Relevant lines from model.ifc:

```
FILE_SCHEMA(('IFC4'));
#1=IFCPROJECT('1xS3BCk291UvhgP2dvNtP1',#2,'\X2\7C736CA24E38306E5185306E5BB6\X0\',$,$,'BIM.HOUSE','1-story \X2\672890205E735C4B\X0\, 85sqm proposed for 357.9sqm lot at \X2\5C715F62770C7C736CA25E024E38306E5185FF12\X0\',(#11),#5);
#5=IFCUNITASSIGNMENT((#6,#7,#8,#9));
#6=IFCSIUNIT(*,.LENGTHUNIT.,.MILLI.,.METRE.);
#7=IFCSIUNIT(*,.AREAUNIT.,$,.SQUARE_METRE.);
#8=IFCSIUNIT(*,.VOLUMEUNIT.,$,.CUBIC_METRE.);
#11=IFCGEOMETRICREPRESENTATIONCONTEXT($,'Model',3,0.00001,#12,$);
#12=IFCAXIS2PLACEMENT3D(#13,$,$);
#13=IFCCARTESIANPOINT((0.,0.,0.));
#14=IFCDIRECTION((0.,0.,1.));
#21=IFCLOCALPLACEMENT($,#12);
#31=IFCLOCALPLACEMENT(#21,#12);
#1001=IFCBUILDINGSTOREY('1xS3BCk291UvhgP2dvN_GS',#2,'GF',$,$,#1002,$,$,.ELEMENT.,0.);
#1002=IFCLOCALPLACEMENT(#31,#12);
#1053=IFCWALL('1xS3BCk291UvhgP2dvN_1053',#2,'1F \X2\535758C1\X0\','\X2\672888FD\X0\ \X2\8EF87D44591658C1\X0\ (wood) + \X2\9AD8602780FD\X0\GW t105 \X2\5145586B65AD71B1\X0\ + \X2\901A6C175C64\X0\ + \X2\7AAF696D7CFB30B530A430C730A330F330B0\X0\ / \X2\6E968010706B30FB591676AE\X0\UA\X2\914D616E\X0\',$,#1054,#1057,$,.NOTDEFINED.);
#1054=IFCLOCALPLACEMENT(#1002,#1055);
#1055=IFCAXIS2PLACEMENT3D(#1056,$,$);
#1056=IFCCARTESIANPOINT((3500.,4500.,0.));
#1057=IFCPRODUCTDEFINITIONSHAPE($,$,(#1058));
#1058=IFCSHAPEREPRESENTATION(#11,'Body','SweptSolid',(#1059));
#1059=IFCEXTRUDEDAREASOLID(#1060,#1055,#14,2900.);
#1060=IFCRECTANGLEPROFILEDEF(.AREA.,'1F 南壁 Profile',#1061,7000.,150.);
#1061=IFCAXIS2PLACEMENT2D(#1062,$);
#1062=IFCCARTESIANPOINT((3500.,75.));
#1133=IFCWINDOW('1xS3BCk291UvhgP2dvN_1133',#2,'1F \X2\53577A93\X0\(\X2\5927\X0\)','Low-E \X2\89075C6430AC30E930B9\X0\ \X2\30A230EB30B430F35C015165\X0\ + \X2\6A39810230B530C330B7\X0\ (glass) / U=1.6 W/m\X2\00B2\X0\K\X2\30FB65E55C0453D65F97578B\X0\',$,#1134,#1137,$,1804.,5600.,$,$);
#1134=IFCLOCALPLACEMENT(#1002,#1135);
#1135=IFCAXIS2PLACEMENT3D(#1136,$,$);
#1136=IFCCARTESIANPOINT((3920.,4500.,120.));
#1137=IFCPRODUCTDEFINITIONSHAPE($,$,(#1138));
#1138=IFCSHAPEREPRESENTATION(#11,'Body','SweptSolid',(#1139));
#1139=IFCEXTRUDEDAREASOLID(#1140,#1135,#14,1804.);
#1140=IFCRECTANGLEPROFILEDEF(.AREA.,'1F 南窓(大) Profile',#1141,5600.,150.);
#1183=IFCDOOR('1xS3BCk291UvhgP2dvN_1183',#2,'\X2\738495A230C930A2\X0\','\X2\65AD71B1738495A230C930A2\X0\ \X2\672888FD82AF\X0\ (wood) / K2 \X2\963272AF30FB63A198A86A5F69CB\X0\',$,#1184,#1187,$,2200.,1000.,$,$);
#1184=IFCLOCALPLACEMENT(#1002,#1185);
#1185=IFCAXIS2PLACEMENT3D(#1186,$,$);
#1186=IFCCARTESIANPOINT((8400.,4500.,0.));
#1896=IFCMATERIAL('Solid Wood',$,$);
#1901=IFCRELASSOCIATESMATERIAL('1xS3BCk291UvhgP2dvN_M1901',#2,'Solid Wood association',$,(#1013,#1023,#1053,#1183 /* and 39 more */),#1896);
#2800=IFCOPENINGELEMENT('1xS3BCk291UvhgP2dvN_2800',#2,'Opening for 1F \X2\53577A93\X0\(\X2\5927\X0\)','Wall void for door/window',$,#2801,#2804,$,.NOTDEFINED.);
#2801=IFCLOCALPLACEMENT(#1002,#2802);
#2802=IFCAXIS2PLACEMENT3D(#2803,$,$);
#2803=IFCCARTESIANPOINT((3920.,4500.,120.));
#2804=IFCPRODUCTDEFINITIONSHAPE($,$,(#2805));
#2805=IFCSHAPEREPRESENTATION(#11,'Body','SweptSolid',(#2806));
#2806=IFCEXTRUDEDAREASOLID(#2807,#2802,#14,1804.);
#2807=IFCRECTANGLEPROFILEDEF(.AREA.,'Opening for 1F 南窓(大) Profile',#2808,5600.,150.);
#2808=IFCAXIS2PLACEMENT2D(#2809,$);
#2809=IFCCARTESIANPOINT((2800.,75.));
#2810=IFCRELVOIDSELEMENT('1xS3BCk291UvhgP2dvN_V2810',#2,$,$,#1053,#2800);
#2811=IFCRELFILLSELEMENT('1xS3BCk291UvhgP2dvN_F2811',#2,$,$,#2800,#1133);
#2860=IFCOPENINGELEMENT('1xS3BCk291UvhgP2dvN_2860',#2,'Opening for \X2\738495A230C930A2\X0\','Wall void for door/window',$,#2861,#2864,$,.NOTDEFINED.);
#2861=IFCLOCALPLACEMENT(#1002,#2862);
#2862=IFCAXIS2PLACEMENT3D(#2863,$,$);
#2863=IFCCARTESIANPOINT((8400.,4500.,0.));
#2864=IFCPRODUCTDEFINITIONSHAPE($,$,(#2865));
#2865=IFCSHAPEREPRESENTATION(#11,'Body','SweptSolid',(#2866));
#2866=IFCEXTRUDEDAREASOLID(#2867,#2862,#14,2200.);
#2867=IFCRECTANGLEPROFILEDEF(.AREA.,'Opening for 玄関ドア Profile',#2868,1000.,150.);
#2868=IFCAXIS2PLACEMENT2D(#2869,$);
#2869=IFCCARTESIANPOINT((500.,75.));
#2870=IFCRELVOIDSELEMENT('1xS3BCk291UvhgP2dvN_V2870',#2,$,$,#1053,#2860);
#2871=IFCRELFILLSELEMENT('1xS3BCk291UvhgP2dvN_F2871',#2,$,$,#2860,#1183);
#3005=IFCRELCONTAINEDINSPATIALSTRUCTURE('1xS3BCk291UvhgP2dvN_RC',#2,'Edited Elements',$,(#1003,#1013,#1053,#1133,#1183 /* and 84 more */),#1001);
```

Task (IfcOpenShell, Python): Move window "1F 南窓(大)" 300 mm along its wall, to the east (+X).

```python
import ifcopenshell
import ifcopenshell.api.geometry
import ifcopenshell.util.placement
import ifcopenshell.util.unit

model = ifcopenshell.open("model.ifc")
unit_scale = ifcopenshell.util.unit.calculate_unit_scale(model)

window = model.by_guid("1xS3BCk291UvhgP2dvN_1133")
opening = window.FillsVoids[0].RelatingOpeningElement
wall = opening.VoidsElements[0].RelatingBuildingElement

wall_matrix = ifcopenshell.util.placement.get_local_placement(wall.ObjectPlacement)
shift = wall_matrix[:3, 0] * 0.3 / unit_scale
before = ifcopenshell.util.placement.get_local_placement(window.ObjectPlacement)[:3, 3].copy()

# The window is not placed relative to its opening, so move both.
for product in (opening, window):
    matrix = ifcopenshell.util.placement.get_local_placement(product.ObjectPlacement)
    matrix[:3, 3] += shift
    ifcopenshell.api.geometry.edit_object_placement(model, product=product, matrix=matrix, is_si=False)

after = ifcopenshell.util.placement.get_local_placement(window.ObjectPlacement)[:3, 3]
print("window moved by", (after - before).round(3) + 0.0)

model.write("model_v2.ifc")
```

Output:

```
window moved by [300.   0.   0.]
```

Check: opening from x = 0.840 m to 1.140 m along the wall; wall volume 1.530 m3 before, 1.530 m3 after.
